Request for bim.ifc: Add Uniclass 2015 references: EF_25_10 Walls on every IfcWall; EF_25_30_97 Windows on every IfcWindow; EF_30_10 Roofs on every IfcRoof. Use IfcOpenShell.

First a look at what the model holds.

```python
import ifcopenshell

model = ifcopenshell.open("bim.ifc")
print(model.schema)
print("classifications:", [c.Name for c in model.by_type("IfcClassification")])
for ifc_class in ("IfcDoor", "IfcRoof", "IfcStair", "IfcWall", "IfcWindow"):
    print(ifc_class, len(model.by_type(ifc_class)))
```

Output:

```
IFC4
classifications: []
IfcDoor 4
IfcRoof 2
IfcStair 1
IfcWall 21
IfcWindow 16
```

```python
import ifcopenshell
import ifcopenshell.api.classification

model = ifcopenshell.open("bim.ifc")

system = ifcopenshell.api.classification.add_classification(model, classification="Uniclass 2015")

codes = {
    "IfcWall": ("EF_25_10", "Walls"),
    "IfcWindow": ("EF_25_30_97", "Windows"),
    "IfcRoof": ("EF_30_10", "Roofs"),
}
for ifc_class, (code, name) in codes.items():
    products = model.by_type(ifc_class)
    ifcopenshell.api.classification.add_reference(
        model, products=products, classification=system, identification=code, name=name
    )
    print(code, len(products))

model.write("bim_v2.ifc")
```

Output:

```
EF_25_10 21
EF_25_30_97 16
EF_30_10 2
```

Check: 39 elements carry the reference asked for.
